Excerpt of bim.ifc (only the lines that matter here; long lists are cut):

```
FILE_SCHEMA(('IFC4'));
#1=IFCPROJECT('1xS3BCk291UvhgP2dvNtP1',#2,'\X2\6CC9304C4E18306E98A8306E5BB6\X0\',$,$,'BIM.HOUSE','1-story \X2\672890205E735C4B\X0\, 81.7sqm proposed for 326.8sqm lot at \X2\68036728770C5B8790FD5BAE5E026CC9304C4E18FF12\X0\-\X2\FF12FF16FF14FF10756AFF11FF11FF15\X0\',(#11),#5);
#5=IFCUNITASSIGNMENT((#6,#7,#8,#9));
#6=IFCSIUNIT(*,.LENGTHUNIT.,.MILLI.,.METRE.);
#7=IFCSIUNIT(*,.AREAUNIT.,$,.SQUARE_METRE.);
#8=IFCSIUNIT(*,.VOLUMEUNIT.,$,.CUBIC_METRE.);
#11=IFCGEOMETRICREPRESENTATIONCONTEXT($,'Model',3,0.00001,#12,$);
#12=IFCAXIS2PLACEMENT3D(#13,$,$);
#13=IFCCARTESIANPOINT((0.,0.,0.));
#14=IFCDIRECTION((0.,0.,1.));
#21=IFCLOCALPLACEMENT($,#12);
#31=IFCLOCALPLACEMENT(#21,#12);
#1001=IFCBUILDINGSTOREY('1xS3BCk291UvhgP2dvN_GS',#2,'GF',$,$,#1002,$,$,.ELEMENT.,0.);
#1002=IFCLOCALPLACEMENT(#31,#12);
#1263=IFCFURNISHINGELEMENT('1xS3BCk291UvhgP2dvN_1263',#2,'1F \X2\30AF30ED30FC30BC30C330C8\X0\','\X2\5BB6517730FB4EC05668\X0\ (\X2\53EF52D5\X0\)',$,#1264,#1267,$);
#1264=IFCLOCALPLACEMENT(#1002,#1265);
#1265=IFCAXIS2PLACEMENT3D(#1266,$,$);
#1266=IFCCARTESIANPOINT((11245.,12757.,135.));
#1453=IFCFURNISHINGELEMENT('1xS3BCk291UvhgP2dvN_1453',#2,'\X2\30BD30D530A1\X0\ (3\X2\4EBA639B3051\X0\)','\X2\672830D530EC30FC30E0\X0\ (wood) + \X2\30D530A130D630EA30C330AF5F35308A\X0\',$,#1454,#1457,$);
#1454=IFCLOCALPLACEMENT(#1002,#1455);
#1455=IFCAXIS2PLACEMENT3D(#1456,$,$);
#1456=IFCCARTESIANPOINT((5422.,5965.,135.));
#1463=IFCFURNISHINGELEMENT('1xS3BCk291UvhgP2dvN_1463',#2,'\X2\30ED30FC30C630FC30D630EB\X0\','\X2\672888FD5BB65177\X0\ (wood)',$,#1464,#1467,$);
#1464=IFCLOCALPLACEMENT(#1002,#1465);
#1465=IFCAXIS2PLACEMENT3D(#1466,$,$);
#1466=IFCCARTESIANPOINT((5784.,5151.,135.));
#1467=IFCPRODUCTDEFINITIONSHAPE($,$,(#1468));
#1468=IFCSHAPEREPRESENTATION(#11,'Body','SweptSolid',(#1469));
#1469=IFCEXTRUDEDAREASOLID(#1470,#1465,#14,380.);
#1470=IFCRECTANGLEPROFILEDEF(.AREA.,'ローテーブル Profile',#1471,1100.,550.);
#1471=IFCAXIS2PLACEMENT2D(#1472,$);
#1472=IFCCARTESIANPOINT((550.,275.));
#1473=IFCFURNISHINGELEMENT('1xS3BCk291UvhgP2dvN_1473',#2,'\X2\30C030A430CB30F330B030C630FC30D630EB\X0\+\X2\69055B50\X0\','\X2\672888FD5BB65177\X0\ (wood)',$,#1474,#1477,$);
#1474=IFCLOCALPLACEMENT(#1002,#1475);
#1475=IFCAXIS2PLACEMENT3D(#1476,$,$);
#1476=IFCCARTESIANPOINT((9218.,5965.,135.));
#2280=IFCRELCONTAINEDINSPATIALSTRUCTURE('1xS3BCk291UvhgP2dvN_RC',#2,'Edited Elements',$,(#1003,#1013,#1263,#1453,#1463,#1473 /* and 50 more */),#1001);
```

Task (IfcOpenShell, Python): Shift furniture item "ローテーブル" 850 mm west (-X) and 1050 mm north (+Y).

```python
import ifcopenshell
import ifcopenshell.api.geometry
import ifcopenshell.util.placement
import ifcopenshell.util.unit

model = ifcopenshell.open("bim.ifc")
unit_scale = ifcopenshell.util.unit.calculate_unit_scale(model)

item = model.by_guid("1xS3BCk291UvhgP2dvN_1463")
matrix = ifcopenshell.util.placement.get_local_placement(item.ObjectPlacement)
matrix[0, 3] -= 0.85 / unit_scale
matrix[1, 3] += 1.05 / unit_scale
ifcopenshell.api.geometry.edit_object_placement(model, product=item, matrix=matrix, is_si=False)

print(ifcopenshell.util.placement.get_local_placement(item.ObjectPlacement).round(3) + 0.0)

model.write("bim_rev.ifc")
```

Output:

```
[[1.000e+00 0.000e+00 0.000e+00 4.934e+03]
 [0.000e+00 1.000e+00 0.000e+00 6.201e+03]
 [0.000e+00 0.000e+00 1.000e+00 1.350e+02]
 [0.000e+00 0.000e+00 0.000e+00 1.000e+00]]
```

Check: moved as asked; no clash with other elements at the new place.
